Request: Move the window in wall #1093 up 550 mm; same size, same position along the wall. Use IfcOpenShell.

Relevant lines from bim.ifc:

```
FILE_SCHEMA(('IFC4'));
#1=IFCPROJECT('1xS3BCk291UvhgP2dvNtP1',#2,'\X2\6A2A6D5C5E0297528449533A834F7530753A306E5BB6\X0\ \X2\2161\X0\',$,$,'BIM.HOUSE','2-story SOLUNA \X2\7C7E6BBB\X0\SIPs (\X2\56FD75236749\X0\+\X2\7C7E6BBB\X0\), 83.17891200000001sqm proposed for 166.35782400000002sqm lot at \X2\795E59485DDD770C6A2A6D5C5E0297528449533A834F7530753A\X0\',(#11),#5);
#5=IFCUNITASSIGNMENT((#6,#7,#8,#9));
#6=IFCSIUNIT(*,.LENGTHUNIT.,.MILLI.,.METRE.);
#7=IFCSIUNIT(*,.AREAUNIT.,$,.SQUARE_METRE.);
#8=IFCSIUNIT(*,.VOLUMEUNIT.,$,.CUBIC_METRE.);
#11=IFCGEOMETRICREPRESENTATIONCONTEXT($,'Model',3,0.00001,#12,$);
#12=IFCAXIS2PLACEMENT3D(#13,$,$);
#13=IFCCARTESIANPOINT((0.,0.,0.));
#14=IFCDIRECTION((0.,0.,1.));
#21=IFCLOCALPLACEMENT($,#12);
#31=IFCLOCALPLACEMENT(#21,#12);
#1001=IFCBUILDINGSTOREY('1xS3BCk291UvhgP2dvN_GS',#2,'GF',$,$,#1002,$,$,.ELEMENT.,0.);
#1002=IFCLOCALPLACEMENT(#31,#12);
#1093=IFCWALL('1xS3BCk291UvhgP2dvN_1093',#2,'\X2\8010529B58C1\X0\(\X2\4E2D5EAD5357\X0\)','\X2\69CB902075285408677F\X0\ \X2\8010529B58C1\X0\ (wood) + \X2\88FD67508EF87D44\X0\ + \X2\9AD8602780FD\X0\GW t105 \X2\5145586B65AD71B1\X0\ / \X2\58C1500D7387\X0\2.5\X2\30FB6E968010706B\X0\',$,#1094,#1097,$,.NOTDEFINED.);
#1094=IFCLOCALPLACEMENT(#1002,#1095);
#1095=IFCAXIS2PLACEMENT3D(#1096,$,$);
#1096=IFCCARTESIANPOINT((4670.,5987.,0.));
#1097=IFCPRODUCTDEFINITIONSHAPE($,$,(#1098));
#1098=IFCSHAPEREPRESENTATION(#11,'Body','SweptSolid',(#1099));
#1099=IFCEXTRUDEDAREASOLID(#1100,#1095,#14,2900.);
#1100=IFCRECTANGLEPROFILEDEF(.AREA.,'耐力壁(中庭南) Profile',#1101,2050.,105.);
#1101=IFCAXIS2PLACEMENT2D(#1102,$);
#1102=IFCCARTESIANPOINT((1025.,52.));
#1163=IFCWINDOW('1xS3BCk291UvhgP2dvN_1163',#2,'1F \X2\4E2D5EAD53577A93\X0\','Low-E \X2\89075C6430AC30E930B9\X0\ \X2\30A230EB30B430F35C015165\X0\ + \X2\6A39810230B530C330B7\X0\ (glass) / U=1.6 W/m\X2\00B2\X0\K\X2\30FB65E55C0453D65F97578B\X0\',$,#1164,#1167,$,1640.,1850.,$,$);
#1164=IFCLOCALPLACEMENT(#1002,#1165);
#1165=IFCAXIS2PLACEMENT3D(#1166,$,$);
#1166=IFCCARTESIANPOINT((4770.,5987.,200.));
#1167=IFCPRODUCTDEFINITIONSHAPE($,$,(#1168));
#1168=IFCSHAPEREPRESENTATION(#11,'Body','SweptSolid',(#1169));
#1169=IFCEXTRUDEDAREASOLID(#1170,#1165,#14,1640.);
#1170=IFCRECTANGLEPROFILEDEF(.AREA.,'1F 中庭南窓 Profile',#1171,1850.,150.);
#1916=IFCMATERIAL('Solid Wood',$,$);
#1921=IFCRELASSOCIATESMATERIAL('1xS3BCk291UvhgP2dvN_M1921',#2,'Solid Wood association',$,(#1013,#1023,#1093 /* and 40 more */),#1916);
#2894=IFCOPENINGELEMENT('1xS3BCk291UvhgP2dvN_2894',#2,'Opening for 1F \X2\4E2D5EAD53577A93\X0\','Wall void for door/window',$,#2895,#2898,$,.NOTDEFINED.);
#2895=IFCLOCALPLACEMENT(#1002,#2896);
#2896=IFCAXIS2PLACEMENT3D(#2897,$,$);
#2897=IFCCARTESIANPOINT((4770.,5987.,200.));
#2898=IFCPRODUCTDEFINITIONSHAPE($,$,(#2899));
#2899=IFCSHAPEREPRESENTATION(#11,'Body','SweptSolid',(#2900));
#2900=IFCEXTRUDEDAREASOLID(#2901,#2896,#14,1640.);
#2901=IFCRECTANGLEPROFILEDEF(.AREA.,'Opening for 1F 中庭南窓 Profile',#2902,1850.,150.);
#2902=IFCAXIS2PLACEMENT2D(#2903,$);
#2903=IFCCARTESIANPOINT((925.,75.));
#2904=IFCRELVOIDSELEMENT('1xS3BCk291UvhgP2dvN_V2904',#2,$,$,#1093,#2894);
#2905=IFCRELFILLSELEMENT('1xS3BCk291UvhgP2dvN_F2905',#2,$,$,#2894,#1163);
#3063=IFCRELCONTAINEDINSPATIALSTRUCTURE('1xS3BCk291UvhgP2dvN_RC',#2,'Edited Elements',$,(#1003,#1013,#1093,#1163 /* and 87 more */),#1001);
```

```python
import numpy as np
import ifcopenshell
import ifcopenshell.api.geometry
import ifcopenshell.util.placement
import ifcopenshell.util.unit

model = ifcopenshell.open("bim.ifc")
unit_scale = ifcopenshell.util.unit.calculate_unit_scale(model)

window = model.by_guid("1xS3BCk291UvhgP2dvN_1163")
opening = window.FillsVoids[0].RelatingOpeningElement
dz = 0.55 / unit_scale

shift = np.array([0.0, 0.0, dz])
# The window is not placed relative to its opening, so move both.
for product in (opening, window):
    matrix = ifcopenshell.util.placement.get_local_placement(product.ObjectPlacement)
    matrix[:3, 3] += shift
    ifcopenshell.api.geometry.edit_object_placement(model, product=product, matrix=matrix, is_si=False)

print(f"moved by {dz * unit_scale:+.3f} m")

model.write("bim_edited.ifc")
```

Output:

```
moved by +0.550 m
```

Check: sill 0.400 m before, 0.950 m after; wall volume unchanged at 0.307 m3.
